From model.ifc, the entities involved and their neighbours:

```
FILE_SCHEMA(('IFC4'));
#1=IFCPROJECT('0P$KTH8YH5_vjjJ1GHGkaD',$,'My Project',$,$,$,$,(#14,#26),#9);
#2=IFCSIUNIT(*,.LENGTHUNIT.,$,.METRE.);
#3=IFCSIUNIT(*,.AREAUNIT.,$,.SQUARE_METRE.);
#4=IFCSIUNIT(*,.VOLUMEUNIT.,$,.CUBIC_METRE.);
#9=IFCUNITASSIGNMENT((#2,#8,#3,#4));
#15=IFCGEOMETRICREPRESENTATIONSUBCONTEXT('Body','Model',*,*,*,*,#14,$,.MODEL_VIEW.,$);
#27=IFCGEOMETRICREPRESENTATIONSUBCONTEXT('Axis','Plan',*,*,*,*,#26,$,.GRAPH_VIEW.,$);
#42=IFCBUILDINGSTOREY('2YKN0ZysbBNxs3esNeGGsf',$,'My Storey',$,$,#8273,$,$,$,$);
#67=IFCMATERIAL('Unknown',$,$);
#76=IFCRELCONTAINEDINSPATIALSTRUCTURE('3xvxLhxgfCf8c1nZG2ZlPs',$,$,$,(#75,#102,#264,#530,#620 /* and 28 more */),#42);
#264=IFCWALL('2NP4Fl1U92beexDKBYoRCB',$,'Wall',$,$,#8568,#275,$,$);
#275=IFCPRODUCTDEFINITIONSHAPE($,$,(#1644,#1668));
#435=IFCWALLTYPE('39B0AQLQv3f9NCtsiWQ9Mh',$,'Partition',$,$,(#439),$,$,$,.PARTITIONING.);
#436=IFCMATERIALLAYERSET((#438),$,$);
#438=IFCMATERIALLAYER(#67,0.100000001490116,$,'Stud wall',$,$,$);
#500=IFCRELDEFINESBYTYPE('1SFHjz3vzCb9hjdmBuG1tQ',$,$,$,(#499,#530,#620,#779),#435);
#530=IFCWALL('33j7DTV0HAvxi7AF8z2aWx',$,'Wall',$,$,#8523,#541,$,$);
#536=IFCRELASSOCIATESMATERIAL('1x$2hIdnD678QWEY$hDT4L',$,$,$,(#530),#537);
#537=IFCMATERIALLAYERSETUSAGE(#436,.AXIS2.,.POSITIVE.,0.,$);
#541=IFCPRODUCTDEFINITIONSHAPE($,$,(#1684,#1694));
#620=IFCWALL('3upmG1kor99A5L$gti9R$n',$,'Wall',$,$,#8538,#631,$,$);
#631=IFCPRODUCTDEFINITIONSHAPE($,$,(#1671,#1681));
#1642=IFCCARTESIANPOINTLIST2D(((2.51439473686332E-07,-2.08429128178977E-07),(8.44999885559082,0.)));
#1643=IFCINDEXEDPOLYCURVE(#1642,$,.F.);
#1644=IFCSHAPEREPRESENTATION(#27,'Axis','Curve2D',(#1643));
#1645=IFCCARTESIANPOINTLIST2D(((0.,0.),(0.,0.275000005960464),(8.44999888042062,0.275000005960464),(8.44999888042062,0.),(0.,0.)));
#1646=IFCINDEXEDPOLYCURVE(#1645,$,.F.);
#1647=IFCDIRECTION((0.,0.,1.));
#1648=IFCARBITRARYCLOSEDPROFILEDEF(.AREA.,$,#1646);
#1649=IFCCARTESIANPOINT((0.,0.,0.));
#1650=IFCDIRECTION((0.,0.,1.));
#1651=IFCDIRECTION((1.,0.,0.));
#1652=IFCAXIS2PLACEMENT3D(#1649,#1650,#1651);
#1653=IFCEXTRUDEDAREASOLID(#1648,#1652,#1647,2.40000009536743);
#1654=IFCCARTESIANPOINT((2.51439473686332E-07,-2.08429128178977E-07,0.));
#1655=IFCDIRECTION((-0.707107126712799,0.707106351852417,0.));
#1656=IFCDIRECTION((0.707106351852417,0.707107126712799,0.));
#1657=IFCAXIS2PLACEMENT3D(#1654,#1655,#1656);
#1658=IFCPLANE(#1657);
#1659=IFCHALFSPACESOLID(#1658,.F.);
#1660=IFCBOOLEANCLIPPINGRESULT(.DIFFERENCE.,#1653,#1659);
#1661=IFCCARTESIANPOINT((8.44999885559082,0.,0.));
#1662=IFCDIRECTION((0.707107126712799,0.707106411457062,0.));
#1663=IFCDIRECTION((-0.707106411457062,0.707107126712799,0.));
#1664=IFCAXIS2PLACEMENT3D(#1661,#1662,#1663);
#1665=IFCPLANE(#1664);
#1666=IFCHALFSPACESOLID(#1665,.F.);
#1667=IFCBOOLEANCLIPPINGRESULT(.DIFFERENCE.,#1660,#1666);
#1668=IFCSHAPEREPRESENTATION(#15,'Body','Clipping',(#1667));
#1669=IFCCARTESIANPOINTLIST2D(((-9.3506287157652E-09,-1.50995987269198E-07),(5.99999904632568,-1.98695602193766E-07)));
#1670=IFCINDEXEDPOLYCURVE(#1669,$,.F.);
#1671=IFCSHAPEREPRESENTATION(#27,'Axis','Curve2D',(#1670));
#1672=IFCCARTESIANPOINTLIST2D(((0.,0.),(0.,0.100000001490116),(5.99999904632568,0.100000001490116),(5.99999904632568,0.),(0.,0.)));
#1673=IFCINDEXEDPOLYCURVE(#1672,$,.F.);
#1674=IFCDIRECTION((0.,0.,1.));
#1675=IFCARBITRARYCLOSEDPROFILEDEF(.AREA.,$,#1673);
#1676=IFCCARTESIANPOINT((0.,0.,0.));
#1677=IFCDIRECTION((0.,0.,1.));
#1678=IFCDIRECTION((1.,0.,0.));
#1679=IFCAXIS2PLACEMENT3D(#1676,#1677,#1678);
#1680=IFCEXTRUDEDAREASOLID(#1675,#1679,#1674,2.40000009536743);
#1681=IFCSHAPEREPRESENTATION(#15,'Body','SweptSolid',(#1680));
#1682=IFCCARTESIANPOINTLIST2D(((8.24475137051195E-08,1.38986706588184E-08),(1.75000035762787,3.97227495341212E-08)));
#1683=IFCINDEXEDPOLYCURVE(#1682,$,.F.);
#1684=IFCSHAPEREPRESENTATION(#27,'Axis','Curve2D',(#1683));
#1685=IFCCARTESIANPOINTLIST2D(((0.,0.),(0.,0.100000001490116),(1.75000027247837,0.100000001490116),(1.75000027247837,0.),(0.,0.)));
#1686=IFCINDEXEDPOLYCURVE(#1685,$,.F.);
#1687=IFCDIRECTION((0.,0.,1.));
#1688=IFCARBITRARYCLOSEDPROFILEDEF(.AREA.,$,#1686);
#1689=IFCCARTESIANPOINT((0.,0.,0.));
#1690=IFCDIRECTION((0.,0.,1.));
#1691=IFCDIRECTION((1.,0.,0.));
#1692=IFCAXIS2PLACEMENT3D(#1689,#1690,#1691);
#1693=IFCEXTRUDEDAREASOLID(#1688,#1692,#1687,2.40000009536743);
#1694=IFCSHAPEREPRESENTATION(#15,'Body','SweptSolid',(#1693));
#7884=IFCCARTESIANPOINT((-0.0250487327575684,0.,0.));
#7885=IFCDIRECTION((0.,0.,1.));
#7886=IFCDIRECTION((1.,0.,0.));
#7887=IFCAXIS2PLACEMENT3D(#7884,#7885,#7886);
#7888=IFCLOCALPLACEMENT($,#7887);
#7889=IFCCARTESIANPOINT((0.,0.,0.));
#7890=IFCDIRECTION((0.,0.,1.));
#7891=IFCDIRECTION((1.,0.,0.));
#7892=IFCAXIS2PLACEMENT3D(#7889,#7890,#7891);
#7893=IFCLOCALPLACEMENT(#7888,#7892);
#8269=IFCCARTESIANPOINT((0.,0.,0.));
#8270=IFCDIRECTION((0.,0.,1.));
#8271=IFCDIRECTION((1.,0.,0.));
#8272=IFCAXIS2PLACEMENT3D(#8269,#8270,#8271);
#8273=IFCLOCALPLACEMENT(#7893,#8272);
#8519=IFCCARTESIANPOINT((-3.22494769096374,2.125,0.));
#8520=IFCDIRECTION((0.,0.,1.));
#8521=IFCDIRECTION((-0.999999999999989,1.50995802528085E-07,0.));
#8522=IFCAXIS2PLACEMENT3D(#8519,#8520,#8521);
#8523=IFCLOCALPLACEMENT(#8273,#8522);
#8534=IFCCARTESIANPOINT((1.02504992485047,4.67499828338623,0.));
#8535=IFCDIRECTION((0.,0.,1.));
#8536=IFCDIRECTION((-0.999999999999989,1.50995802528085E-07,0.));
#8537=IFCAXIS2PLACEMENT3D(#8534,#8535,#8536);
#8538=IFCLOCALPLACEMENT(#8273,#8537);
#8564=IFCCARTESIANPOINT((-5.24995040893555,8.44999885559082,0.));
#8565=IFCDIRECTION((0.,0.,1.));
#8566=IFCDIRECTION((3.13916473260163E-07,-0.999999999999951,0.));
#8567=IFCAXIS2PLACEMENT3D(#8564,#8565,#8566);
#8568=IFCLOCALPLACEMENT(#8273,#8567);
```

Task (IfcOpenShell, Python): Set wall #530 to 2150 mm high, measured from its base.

```python
import ifcopenshell
import ifcopenshell.geom
import ifcopenshell.util.representation
import ifcopenshell.util.shape
import ifcopenshell.util.unit

model = ifcopenshell.open("model.ifc")
unit_scale = ifcopenshell.util.unit.calculate_unit_scale(model)
settings = ifcopenshell.geom.settings()


def volume(element):
    """Net volume in cubic metres, openings subtracted."""
    shape = ifcopenshell.geom.create_shape(settings, element)
    return ifcopenshell.util.shape.get_volume(shape.geometry)


wall = model.by_id(530)
before = volume(wall)

body = ifcopenshell.util.representation.get_representation(wall, "Model", "Body")
solid = body.Items[0]
old_height = solid.Depth
solid.Depth = 2.15 / unit_scale
after = volume(wall)

print(f"height {old_height:g} -> {solid.Depth:g}, volume {before:.3f} -> {after:.3f} m3")

model.write("model_rev.ifc")
```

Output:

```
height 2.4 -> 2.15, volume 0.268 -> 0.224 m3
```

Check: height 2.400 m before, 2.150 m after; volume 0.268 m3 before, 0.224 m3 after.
